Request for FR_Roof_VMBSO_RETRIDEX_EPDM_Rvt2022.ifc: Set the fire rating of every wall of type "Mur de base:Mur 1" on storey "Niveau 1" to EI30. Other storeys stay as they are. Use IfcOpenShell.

First a look at what the model holds.

```python
import ifcopenshell
import ifcopenshell.util.element

model = ifcopenshell.open("FR_Roof_VMBSO_RETRIDEX_EPDM_Rvt2022.ifc")
print(model.schema)
storey = next(s for s in model.by_type("IfcBuildingStorey") if s.Name == "Niveau 1")
walls = [e for e in ifcopenshell.util.element.get_decomposition(storey) if e.is_a("IfcWall")]
seen = {}
for e in walls:
    element_type = ifcopenshell.util.element.get_type(e)
    key = (element_type.Name if element_type != e and element_type else None, ifcopenshell.util.element.get_pset(e, "Pset_WallCommon", "FireRating"))
    seen[key] = seen.get(key, 0) + 1
for (name, value), count in sorted(seen.items(), key=str):
    print(count, "x", name, "|", value)
```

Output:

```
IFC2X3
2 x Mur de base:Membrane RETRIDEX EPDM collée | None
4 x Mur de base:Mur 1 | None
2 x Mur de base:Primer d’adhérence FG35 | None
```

```python
import ifcopenshell
import ifcopenshell.api.pset
import ifcopenshell.util.element

model = ifcopenshell.open("FR_Roof_VMBSO_RETRIDEX_EPDM_Rvt2022.ifc")

storey = next(s for s in model.by_type("IfcBuildingStorey") if s.Name == "Niveau 1")
walls = [e for e in ifcopenshell.util.element.get_decomposition(storey) if e.is_a("IfcWall")]

count = 0
for e in walls:
    element_type = ifcopenshell.util.element.get_type(e)
    if element_type in (None, e) or element_type.Name != "Mur de base:Mur 1":
        continue
    # add_pset returns the element's existing set when there is one.
    pset = ifcopenshell.api.pset.add_pset(model, product=e, name="Pset_WallCommon")
    ifcopenshell.api.pset.edit_pset(model, pset=pset, properties={"FireRating": "EI30"})
    count += 1

print(count, "walls updated")

model.write("FR_Roof_VMBSO_RETRIDEX_EPDM_Rvt2022_v2.ifc")
```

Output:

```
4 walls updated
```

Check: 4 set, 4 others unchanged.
